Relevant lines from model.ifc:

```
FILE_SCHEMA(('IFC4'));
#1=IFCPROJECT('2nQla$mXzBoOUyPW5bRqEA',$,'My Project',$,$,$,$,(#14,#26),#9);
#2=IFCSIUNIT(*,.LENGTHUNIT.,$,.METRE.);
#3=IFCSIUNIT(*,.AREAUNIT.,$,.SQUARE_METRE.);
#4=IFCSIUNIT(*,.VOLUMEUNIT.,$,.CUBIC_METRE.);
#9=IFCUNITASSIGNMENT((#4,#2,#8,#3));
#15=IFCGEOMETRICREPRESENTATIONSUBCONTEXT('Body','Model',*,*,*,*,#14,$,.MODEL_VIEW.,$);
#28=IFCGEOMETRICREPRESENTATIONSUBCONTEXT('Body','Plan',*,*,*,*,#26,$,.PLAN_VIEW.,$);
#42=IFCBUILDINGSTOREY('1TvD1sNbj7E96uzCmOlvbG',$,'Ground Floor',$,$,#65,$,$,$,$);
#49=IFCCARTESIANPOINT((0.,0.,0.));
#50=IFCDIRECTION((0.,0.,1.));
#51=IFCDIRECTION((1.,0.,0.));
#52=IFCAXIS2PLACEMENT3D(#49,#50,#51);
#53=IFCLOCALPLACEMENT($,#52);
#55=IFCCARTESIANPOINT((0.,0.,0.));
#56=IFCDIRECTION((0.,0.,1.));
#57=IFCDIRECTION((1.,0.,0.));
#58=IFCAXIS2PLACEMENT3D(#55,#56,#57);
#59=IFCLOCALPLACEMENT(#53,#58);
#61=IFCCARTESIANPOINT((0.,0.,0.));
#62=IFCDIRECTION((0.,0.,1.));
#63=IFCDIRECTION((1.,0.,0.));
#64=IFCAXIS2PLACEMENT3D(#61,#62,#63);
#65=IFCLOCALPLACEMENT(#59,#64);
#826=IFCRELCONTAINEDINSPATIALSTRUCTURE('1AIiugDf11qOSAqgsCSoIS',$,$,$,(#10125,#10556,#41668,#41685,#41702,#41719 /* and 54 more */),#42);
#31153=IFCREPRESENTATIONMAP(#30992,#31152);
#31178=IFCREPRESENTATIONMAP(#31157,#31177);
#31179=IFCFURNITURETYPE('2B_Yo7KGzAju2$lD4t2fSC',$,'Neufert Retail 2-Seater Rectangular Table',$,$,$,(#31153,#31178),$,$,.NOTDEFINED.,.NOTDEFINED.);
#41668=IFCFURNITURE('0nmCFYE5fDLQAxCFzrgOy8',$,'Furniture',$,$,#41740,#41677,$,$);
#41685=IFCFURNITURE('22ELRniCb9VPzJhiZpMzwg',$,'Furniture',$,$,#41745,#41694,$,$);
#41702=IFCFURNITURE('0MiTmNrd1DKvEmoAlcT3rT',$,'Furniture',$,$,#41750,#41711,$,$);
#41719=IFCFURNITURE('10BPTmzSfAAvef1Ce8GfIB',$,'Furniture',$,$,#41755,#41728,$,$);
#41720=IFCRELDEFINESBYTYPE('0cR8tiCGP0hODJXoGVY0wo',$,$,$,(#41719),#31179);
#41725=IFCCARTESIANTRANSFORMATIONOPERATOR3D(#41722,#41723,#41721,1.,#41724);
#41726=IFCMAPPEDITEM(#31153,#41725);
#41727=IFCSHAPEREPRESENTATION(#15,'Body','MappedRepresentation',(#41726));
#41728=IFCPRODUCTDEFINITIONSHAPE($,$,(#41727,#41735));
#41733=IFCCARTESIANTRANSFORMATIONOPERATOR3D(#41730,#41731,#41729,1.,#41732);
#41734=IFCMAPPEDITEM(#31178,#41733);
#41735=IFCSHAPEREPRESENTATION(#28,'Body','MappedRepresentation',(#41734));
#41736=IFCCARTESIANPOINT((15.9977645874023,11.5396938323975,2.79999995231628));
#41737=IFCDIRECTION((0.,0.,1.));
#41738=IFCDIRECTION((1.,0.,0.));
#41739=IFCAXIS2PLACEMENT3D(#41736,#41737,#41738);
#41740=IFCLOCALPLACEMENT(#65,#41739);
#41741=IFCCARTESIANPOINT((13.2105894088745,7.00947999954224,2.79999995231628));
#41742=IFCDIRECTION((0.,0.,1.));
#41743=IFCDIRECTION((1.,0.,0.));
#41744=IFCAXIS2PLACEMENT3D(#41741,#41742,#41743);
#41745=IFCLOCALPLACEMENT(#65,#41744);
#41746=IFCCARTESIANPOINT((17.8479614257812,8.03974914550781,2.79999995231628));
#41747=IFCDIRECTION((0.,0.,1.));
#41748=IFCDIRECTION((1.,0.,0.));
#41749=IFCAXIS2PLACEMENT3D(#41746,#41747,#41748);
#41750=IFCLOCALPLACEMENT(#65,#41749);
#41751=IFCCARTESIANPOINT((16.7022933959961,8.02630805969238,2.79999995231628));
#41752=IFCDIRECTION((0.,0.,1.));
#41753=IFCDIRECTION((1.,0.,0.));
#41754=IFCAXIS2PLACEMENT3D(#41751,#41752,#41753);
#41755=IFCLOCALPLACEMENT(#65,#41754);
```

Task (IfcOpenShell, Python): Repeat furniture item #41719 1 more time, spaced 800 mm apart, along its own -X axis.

```python
import ifcopenshell
import ifcopenshell.api.geometry
import ifcopenshell.api.root
import ifcopenshell.util.element
import ifcopenshell.util.placement
import ifcopenshell.util.unit

model = ifcopenshell.open("model.ifc")
unit_scale = ifcopenshell.util.unit.calculate_unit_scale(model)

source = model.by_guid("10BPTmzSfAAvef1Ce8GfIB")
base = ifcopenshell.util.placement.get_local_placement(source.ObjectPlacement)
step = -base[:3, 0] * 0.8 / unit_scale

for i in range(1, 2):
    copy = ifcopenshell.api.root.copy_class(model, product=source)
    copy.Representation = ifcopenshell.util.element.copy_deep(
        model, source.Representation, exclude=["IfcGeometricRepresentationContext", "IfcRepresentationMap"]
    )
    matrix = base.copy()
    matrix[:3, 3] += i * step
    print("added at", matrix[:3, 3].round(3) + 0.0)
    ifcopenshell.api.geometry.edit_object_placement(model, product=copy, matrix=matrix, is_si=False)

model.write("model_rev.ifc")
```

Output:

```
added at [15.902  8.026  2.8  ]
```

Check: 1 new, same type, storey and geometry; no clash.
